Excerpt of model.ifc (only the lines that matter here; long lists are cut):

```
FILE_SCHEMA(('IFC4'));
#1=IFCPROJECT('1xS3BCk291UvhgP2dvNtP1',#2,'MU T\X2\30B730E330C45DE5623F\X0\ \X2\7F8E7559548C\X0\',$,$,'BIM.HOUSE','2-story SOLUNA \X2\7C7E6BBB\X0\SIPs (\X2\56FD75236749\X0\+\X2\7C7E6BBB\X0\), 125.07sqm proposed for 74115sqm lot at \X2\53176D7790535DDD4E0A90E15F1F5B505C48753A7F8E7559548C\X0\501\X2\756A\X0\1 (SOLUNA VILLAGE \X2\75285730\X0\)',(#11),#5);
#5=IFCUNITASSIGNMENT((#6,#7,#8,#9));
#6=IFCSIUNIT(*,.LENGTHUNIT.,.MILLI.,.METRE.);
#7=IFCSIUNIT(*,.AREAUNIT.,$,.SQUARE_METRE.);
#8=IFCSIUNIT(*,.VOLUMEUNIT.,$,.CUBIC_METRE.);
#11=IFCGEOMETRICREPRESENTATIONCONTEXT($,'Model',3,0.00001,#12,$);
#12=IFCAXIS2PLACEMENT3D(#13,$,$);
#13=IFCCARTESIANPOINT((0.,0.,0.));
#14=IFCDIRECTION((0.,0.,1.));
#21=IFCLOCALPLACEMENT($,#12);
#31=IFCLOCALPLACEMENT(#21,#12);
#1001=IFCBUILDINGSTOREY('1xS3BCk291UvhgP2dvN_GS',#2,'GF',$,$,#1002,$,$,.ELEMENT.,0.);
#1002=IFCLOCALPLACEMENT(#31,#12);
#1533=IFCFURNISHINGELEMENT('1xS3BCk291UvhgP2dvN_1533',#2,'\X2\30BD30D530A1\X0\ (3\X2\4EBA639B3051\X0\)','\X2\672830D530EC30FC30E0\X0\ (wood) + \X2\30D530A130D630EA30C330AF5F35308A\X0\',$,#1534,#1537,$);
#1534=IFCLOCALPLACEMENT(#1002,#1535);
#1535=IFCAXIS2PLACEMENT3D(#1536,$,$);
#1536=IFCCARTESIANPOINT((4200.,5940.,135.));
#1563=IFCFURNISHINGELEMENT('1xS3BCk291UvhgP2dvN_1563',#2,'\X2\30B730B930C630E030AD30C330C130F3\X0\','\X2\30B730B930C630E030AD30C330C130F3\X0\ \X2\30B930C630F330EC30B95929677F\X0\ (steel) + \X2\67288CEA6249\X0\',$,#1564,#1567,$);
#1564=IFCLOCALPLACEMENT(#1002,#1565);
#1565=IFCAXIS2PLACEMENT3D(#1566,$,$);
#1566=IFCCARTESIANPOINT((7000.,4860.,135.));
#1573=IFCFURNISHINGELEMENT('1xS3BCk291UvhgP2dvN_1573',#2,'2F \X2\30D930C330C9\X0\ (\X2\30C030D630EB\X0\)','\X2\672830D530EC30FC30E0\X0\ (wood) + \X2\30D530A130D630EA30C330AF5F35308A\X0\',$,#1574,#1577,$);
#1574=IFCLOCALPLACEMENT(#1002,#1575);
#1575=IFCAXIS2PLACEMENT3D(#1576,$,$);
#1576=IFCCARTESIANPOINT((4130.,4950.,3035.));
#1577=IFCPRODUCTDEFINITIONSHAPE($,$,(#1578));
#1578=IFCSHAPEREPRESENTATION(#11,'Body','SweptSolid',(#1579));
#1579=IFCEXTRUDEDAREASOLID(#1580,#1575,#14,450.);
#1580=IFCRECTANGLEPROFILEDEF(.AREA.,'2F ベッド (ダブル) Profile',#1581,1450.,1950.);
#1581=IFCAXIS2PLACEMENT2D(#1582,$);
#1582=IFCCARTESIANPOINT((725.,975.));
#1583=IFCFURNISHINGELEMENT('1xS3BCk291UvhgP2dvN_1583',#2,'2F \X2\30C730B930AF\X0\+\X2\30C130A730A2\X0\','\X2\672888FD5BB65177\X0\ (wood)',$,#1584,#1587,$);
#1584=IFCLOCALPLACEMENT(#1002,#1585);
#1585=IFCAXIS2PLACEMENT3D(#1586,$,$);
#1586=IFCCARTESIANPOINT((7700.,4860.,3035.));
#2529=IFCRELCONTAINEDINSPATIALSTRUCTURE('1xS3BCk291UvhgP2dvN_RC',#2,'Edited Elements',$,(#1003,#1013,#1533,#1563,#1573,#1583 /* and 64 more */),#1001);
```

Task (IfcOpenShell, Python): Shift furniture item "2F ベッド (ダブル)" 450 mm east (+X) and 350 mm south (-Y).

```python
import ifcopenshell
import ifcopenshell.api.geometry
import ifcopenshell.util.placement
import ifcopenshell.util.unit

model = ifcopenshell.open("model.ifc")
unit_scale = ifcopenshell.util.unit.calculate_unit_scale(model)

item = model.by_id(1573)
matrix = ifcopenshell.util.placement.get_local_placement(item.ObjectPlacement)
matrix[0, 3] += 0.45 / unit_scale
matrix[1, 3] -= 0.35 / unit_scale
ifcopenshell.api.geometry.edit_object_placement(model, product=item, matrix=matrix, is_si=False)

print(ifcopenshell.util.placement.get_local_placement(item.ObjectPlacement).round(3) + 0.0)

model.write("model_edited.ifc")
```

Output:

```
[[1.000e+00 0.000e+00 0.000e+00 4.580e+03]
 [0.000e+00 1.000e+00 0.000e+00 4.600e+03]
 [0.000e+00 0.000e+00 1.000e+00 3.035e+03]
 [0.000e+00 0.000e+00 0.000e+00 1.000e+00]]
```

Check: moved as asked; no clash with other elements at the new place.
